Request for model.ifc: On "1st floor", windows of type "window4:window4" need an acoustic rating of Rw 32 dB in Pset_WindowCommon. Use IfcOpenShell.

First a look at what the model holds.

```python
import ifcopenshell
import ifcopenshell.util.element

model = ifcopenshell.open("model.ifc")
print(model.schema)
storey = next(s for s in model.by_type("IfcBuildingStorey") if s.Name == "1st floor")
windows = [e for e in ifcopenshell.util.element.get_decomposition(storey) if e.is_a("IfcWindow")]
seen = {}
for e in windows:
    element_type = ifcopenshell.util.element.get_type(e)
    key = (element_type.Name if element_type != e and element_type else None, ifcopenshell.util.element.get_pset(e, "Pset_WindowCommon", "AcousticRating"))
    seen[key] = seen.get(key, 0) + 1
for (name, value), count in sorted(seen.items(), key=str):
    print(count, "x", name, "|", value)
```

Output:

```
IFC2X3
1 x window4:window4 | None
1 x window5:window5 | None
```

```python
import ifcopenshell
import ifcopenshell.api.pset
import ifcopenshell.util.element

model = ifcopenshell.open("model.ifc")

storey = next(s for s in model.by_type("IfcBuildingStorey") if s.Name == "1st floor")
windows = [e for e in ifcopenshell.util.element.get_decomposition(storey) if e.is_a("IfcWindow")]

count = 0
for e in windows:
    element_type = ifcopenshell.util.element.get_type(e)
    if element_type in (None, e) or element_type.Name != "window4:window4":
        continue
    # add_pset returns the element's existing set when there is one.
    pset = ifcopenshell.api.pset.add_pset(model, product=e, name="Pset_WindowCommon")
    ifcopenshell.api.pset.edit_pset(model, pset=pset, properties={"AcousticRating": "Rw 32 dB"})
    count += 1

print(count, "windows updated")

model.write("model-out.ifc")
```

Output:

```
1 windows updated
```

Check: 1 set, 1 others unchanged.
